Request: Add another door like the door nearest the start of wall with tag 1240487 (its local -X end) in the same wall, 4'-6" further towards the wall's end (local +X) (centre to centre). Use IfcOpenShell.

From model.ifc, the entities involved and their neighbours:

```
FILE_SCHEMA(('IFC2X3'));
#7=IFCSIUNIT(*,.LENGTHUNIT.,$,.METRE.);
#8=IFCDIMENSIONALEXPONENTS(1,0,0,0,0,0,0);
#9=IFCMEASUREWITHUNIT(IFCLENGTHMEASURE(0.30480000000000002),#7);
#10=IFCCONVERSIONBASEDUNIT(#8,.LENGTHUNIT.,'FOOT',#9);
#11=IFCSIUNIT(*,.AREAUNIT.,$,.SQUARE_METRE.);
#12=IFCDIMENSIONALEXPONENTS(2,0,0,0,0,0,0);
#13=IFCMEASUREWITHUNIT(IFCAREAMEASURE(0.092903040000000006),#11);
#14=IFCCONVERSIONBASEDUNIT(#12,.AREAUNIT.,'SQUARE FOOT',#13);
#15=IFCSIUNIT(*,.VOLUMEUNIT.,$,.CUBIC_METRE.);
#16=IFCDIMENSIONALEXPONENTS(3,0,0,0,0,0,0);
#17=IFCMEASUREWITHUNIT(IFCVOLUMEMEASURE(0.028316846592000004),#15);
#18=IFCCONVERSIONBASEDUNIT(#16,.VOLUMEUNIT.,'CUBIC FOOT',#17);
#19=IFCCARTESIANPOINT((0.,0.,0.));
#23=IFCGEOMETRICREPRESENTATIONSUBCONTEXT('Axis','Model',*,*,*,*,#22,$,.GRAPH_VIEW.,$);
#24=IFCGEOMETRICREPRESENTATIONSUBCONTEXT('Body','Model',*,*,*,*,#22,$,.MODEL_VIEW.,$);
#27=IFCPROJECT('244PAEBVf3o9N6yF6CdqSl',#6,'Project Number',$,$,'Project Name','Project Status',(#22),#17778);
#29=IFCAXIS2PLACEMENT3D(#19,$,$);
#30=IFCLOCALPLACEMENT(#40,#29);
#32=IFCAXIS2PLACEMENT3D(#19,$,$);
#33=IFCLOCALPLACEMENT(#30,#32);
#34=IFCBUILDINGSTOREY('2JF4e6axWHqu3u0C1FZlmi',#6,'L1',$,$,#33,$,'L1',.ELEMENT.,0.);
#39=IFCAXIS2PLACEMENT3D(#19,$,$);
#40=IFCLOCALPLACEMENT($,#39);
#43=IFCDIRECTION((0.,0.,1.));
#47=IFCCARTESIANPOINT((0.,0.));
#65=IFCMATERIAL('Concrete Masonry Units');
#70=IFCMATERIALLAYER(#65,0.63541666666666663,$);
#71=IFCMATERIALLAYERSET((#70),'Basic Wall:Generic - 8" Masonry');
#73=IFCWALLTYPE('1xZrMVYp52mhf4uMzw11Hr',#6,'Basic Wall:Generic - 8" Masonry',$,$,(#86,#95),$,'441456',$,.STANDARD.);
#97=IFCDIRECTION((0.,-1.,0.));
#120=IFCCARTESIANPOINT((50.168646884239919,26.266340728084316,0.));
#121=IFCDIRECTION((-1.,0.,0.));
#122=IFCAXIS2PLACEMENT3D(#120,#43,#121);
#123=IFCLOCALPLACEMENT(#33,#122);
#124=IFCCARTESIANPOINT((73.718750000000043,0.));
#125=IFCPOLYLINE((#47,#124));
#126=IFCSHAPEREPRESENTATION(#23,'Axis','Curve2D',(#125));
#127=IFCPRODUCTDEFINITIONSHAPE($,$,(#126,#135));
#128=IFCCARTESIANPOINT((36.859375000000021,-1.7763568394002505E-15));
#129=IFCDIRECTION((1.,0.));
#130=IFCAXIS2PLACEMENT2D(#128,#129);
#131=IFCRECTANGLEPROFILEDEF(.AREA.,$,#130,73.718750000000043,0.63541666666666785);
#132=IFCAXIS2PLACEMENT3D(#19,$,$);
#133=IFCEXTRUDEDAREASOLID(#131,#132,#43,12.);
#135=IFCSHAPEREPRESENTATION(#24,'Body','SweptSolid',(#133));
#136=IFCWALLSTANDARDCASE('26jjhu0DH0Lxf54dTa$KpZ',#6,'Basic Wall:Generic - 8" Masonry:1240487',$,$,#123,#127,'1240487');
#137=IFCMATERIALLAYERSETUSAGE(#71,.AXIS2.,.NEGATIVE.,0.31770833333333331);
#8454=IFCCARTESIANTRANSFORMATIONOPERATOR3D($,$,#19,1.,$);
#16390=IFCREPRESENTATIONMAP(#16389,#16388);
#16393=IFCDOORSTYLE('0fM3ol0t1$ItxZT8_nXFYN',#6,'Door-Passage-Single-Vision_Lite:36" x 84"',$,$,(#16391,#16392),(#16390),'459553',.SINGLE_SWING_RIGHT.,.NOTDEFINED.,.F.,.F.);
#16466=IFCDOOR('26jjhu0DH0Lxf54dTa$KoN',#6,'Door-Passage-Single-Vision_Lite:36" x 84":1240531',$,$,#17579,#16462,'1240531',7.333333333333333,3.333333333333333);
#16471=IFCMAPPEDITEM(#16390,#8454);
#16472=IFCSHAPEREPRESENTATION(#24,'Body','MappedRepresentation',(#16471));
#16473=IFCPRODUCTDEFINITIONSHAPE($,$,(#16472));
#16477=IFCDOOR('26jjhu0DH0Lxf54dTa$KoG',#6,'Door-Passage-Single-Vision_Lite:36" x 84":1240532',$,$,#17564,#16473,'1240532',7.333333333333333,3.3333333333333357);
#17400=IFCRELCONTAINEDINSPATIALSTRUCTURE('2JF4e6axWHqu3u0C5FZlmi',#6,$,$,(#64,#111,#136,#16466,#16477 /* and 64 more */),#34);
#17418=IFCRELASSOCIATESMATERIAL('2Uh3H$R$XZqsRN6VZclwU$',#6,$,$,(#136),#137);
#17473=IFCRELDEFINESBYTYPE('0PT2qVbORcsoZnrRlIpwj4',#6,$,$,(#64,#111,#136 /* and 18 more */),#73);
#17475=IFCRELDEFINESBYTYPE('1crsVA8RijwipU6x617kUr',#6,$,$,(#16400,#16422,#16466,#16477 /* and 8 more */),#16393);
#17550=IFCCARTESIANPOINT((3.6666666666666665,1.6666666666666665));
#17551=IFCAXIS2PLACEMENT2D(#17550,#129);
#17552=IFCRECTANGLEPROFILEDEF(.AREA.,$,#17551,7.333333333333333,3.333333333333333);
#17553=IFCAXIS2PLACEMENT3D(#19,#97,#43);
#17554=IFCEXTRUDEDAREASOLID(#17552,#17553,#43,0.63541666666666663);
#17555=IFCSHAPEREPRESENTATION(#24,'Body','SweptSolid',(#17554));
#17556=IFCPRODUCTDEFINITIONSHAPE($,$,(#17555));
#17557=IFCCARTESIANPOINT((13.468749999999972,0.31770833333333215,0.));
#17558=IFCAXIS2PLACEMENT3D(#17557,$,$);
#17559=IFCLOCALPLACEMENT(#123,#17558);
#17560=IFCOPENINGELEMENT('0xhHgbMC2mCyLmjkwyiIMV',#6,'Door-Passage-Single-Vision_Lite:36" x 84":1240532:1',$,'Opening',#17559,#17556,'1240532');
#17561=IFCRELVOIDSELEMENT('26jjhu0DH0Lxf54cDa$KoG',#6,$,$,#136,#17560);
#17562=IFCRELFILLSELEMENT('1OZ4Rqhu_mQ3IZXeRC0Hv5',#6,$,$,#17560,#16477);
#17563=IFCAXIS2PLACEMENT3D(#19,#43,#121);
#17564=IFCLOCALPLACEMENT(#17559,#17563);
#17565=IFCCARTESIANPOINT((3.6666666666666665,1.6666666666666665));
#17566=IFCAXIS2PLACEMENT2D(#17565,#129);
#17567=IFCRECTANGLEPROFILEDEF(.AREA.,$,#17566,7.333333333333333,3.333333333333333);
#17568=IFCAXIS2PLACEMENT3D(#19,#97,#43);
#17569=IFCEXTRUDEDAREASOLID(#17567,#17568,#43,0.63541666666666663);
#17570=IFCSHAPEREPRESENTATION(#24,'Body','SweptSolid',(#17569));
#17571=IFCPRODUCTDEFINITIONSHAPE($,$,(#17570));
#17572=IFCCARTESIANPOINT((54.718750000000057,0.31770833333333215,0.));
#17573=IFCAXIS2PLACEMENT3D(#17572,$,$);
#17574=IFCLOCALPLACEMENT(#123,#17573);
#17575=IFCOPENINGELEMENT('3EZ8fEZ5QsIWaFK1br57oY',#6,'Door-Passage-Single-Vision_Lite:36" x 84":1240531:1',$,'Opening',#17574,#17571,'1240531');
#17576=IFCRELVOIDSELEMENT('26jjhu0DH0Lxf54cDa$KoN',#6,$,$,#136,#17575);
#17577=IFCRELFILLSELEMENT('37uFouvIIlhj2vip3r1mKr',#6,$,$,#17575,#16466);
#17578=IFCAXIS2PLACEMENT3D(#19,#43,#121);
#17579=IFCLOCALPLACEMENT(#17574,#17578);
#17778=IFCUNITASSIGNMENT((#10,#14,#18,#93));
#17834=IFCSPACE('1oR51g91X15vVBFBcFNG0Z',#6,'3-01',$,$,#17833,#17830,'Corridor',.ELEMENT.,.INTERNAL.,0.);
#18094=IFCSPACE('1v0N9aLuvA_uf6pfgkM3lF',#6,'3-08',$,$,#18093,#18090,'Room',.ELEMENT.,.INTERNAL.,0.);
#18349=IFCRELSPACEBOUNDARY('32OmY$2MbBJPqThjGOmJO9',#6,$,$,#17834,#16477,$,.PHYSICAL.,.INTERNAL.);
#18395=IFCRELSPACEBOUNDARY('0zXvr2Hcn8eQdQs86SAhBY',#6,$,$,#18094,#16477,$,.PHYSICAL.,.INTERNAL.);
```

```python
import ifcopenshell
import ifcopenshell.api.feature
import ifcopenshell.api.geometry
import ifcopenshell.api.root
import ifcopenshell.geom
import ifcopenshell.util.element
import ifcopenshell.util.placement
import ifcopenshell.util.shape
import ifcopenshell.util.unit

model = ifcopenshell.open("model.ifc")
unit_scale = ifcopenshell.util.unit.calculate_unit_scale(model)
settings = ifcopenshell.geom.settings()


def volume(element):
    """Net volume in cubic metres, openings subtracted."""
    shape = ifcopenshell.geom.create_shape(settings, element)
    return ifcopenshell.util.shape.get_volume(shape.geometry)


def reuse_history(source, copy):
    """copy_class also copies each property set's owner history, people and application; keep the originals."""
    for rel in copy.IsDefinedBy:
        if rel.is_a("IfcRelDefinesByProperties") and (history := rel.RelatingPropertyDefinition.OwnerHistory):
            rel.RelatingPropertyDefinition.OwnerHistory = source.OwnerHistory
            ifcopenshell.util.element.remove_deep2(model, history)


door = model.by_guid("26jjhu0DH0Lxf54dTa$KoG")
opening = door.FillsVoids[0].RelatingOpeningElement
wall = opening.VoidsElements[0].RelatingBuildingElement
before = volume(wall)
shift = ifcopenshell.util.placement.get_local_placement(wall.ObjectPlacement)[:3, 0] * 54 * 0.0254 / unit_scale

# copy_class copies the void relationship, type, container and properties, but no geometry.
new_opening = ifcopenshell.api.root.copy_class(model, product=opening)
new_opening.Representation = ifcopenshell.util.element.copy_deep(
    model, opening.Representation, exclude=["IfcGeometricRepresentationContext", "IfcRepresentationMap"]
)
new_opening.Name = 'Door-Passage-Single-Vision_Lite:36" x 84"'
new_opening.Tag = None
new_door = ifcopenshell.api.root.copy_class(model, product=door)
new_door.Representation = ifcopenshell.util.element.copy_deep(
    model, door.Representation, exclude=["IfcGeometricRepresentationContext", "IfcRepresentationMap"]
)
new_door.Name = 'Door-Passage-Single-Vision_Lite:36" x 84"'
new_door.Tag = None
reuse_history(door, new_door)
fills = ifcopenshell.api.feature.add_filling(model, opening=new_opening, element=new_door)
fills.OwnerHistory = new_door.OwnerHistory  # required in IFC2X3

for old, new in ((opening, new_opening), (door, new_door)):
    matrix = ifcopenshell.util.placement.get_local_placement(old.ObjectPlacement)
    matrix[:3, 3] += shift
    ifcopenshell.api.geometry.edit_object_placement(model, product=new, matrix=matrix, is_si=False)

after = volume(wall)

print(f"wall volume {before:.3f} -> {after:.3f} m3")

model.write("model_v2.ifc")
```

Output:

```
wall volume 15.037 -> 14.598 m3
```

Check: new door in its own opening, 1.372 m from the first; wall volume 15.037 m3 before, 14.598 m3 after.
